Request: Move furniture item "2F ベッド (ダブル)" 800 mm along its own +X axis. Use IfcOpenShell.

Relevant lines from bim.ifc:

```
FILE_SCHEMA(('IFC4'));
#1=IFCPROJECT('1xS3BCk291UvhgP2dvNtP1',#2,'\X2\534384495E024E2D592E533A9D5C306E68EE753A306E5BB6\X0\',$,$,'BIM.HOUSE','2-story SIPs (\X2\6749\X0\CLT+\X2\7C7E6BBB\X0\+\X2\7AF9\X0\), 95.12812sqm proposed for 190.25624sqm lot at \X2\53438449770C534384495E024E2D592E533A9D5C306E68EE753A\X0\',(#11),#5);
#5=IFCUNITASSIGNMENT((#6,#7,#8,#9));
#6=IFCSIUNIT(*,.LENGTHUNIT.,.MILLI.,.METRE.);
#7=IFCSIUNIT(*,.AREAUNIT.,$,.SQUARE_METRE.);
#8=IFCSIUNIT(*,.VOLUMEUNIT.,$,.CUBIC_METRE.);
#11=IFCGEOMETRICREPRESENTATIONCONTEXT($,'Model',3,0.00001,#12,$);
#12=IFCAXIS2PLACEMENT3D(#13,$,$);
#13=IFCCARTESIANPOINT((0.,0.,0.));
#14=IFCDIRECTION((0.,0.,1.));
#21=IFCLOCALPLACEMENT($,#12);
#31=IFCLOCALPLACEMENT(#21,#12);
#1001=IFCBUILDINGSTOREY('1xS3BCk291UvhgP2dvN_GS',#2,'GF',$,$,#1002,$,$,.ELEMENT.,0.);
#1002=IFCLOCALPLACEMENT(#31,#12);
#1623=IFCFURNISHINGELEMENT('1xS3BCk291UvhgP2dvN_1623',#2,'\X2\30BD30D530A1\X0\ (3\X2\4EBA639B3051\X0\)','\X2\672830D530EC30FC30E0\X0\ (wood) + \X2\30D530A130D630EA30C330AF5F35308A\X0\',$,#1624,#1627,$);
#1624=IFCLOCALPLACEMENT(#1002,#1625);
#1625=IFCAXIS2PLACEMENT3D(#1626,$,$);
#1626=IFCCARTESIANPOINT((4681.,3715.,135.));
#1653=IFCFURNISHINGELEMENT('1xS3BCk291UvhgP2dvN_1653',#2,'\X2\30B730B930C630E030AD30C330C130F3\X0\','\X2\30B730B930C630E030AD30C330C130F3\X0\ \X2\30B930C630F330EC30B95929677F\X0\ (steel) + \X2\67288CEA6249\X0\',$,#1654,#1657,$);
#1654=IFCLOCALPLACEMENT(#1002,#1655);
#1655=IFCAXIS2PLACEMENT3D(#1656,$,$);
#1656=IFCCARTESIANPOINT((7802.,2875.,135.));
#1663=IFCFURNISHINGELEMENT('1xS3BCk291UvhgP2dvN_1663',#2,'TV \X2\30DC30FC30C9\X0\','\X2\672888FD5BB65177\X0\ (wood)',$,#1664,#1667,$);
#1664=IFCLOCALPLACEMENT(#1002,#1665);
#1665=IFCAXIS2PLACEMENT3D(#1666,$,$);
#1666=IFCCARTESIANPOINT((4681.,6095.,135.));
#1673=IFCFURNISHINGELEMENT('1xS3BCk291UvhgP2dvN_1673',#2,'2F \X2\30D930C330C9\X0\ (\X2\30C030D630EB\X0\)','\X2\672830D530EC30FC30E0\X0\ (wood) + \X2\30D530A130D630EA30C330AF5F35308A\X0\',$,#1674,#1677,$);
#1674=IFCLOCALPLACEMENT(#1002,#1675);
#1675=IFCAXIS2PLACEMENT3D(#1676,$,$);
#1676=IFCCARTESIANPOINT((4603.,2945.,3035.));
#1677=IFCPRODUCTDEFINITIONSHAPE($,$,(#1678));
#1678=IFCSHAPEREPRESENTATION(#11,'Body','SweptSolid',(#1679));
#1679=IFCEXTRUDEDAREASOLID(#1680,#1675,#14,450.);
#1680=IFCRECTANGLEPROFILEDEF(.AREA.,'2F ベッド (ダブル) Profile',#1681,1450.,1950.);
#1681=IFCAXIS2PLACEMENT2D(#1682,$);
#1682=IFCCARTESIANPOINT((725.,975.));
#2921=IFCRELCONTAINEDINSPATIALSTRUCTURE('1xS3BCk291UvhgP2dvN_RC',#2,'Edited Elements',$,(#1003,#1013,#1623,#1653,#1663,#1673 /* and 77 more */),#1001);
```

```python
import ifcopenshell
import ifcopenshell.api.geometry
import ifcopenshell.util.placement
import ifcopenshell.util.unit

model = ifcopenshell.open("bim.ifc")
unit_scale = ifcopenshell.util.unit.calculate_unit_scale(model)

item = model.by_guid("1xS3BCk291UvhgP2dvN_1673")
matrix = ifcopenshell.util.placement.get_local_placement(item.ObjectPlacement)
matrix[:3, 3] += matrix[:3, 0] * 0.8 / unit_scale
ifcopenshell.api.geometry.edit_object_placement(model, product=item, matrix=matrix, is_si=False)

print(ifcopenshell.util.placement.get_local_placement(item.ObjectPlacement).round(3) + 0.0)

model.write("bim_rev.ifc")
```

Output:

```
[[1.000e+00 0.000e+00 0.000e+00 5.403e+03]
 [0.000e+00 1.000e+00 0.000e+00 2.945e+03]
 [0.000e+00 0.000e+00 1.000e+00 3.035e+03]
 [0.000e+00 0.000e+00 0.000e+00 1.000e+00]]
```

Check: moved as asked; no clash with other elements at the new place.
